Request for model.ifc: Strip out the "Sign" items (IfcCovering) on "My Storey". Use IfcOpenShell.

First a look at what the model holds.

```python
import ifcopenshell
import ifcopenshell.util.element

model = ifcopenshell.open("model.ifc")
print(model.schema)
storey = next(s for s in model.by_type("IfcBuildingStorey") if s.Name == "My Storey")
coverings = [e for e in ifcopenshell.util.element.get_decomposition(storey) if e.is_a("IfcCovering")]
seen = {}
for e in coverings:
    element_type = ifcopenshell.util.element.get_type(e)
    name = element_type.Name if element_type not in (None, e) else None
    seen[name] = seen.get(name, 0) + 1
for name, count in sorted(seen.items(), key=str):
    print(count, "x", name)
```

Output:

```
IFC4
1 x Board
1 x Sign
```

```python
import ifcopenshell
import ifcopenshell.api.root
import ifcopenshell.util.element

model = ifcopenshell.open("model.ifc")

storey = next(s for s in model.by_type("IfcBuildingStorey") if s.Name == "My Storey")
coverings = [e for e in ifcopenshell.util.element.get_decomposition(storey) if e.is_a("IfcCovering")]
targets = [e for e in coverings if (t := ifcopenshell.util.element.get_type(e)) not in (None, e) and t.Name == "Sign"]

for e in targets:
    ifcopenshell.api.root.remove_product(model, product=e)
print(len(targets), "removed")

model.write("model_rev.ifc")
```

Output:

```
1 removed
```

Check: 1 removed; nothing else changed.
